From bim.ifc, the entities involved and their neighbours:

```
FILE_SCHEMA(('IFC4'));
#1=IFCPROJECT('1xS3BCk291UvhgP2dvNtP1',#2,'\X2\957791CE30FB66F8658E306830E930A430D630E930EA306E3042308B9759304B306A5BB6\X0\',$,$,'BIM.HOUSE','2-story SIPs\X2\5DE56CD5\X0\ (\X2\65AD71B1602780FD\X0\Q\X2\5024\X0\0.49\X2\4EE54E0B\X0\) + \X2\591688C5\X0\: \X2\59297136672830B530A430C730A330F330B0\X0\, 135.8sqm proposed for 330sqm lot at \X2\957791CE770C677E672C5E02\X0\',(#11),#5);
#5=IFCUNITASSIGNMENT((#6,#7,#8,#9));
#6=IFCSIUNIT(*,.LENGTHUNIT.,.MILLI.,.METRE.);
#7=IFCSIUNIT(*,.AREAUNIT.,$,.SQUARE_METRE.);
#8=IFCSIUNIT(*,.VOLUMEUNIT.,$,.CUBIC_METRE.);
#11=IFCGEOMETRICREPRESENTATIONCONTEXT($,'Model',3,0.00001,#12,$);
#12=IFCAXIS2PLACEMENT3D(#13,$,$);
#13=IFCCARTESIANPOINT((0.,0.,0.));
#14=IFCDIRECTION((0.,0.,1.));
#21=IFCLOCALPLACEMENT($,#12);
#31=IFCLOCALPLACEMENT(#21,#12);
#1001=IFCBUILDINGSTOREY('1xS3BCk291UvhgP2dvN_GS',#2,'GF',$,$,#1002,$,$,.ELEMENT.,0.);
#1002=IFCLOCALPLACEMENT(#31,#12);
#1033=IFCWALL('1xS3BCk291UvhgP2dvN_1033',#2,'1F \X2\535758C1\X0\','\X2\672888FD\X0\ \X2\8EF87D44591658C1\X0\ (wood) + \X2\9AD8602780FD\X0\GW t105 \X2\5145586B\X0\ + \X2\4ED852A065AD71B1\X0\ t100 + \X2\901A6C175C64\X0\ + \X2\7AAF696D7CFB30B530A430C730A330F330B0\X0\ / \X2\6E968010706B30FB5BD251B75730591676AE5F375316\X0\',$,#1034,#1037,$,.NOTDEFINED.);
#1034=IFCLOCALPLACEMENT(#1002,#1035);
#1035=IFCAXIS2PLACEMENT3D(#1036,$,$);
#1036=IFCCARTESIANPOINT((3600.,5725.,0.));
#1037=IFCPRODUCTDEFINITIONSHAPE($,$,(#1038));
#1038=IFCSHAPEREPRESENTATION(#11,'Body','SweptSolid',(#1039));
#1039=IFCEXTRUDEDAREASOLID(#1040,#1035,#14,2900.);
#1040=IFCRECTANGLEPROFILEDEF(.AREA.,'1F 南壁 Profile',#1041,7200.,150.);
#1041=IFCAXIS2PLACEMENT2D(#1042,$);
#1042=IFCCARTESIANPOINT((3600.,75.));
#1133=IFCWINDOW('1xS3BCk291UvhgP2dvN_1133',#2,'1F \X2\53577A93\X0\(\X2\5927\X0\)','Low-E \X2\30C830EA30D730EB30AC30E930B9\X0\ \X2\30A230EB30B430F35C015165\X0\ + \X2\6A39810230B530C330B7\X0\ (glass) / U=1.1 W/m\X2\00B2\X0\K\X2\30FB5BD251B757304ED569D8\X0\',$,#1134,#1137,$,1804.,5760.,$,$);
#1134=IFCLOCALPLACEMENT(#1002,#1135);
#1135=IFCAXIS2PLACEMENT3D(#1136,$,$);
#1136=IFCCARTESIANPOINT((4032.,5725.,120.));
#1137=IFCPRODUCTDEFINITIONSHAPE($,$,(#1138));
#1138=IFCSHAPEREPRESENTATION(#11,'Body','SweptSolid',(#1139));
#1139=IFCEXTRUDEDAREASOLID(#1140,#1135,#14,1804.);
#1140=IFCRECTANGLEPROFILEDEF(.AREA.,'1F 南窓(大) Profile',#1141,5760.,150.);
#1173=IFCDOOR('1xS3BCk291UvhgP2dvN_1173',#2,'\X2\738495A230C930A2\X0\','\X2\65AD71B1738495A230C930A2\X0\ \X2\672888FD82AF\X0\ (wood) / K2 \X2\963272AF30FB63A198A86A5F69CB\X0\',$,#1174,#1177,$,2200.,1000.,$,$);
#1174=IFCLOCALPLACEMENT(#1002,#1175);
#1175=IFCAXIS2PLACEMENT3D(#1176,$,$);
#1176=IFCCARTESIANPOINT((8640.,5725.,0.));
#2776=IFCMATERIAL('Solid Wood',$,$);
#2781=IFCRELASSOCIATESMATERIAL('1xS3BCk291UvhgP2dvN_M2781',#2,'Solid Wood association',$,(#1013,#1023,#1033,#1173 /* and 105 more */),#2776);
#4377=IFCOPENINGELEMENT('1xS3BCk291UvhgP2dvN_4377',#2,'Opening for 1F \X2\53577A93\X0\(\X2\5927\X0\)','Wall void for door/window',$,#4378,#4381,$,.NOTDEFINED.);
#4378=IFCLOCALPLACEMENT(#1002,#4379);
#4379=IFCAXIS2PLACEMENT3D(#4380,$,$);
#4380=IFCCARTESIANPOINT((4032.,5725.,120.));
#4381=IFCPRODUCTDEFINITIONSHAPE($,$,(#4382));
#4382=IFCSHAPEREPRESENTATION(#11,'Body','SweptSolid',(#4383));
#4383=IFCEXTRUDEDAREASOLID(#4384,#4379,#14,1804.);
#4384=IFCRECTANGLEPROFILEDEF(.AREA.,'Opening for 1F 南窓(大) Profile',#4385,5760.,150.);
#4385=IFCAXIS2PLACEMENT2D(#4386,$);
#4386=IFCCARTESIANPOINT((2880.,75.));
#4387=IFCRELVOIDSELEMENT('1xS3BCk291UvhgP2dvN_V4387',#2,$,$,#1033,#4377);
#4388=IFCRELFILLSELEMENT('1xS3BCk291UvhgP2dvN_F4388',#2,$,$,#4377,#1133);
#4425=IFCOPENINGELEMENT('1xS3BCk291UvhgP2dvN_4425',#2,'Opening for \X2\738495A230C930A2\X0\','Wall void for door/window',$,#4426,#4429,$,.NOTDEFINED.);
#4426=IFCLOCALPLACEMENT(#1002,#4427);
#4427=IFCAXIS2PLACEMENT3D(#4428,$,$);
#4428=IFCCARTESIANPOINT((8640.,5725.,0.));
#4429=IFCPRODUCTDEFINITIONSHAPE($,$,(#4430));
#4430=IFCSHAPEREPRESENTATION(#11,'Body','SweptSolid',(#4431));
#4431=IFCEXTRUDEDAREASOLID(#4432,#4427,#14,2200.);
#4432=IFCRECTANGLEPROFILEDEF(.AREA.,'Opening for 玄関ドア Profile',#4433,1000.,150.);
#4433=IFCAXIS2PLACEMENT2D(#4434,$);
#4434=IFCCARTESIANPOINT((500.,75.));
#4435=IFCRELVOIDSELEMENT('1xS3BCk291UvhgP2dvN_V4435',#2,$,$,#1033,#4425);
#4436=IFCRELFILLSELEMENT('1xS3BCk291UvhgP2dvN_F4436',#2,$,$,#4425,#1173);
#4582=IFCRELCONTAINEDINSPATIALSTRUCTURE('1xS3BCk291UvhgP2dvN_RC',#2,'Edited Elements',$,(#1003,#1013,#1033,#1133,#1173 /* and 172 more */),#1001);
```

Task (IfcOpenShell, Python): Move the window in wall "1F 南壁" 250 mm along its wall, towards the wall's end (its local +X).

```python
import ifcopenshell
import ifcopenshell.api.geometry
import ifcopenshell.util.placement
import ifcopenshell.util.unit

model = ifcopenshell.open("bim.ifc")
unit_scale = ifcopenshell.util.unit.calculate_unit_scale(model)

window = model.by_id(1133)
opening = window.FillsVoids[0].RelatingOpeningElement
wall = opening.VoidsElements[0].RelatingBuildingElement

wall_matrix = ifcopenshell.util.placement.get_local_placement(wall.ObjectPlacement)
shift = wall_matrix[:3, 0] * 0.25 / unit_scale
before = ifcopenshell.util.placement.get_local_placement(window.ObjectPlacement)[:3, 3].copy()

# The window is not placed relative to its opening, so move both.
for product in (opening, window):
    matrix = ifcopenshell.util.placement.get_local_placement(product.ObjectPlacement)
    matrix[:3, 3] += shift
    ifcopenshell.api.geometry.edit_object_placement(model, product=product, matrix=matrix, is_si=False)

after = ifcopenshell.util.placement.get_local_placement(window.ObjectPlacement)[:3, 3]
print("window moved by", (after - before).round(3) + 0.0)

model.write("bim_rev.ifc")
```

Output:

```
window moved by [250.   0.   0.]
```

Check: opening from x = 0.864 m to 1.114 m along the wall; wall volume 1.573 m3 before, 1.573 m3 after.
